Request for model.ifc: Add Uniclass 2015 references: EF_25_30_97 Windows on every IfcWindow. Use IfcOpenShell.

First a look at what the model holds.

```python
import ifcopenshell

model = ifcopenshell.open("model.ifc")
print(model.schema)
print("classifications:", [c.Name for c in model.by_type("IfcClassification")])
for ifc_class in ("IfcDoor", "IfcRoof", "IfcStair", "IfcWall", "IfcWindow"):
    print(ifc_class, len(model.by_type(ifc_class)))
```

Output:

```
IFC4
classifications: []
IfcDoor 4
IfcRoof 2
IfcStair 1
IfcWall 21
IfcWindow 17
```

```python
import ifcopenshell
import ifcopenshell.api.classification

model = ifcopenshell.open("model.ifc")

system = ifcopenshell.api.classification.add_classification(model, classification="Uniclass 2015")

codes = {
    "IfcWindow": ("EF_25_30_97", "Windows"),
}
for ifc_class, (code, name) in codes.items():
    products = model.by_type(ifc_class)
    ifcopenshell.api.classification.add_reference(
        model, products=products, classification=system, identification=code, name=name
    )
    print(code, len(products))

model.write("model_edited.ifc")
```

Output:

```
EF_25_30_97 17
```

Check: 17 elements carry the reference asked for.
